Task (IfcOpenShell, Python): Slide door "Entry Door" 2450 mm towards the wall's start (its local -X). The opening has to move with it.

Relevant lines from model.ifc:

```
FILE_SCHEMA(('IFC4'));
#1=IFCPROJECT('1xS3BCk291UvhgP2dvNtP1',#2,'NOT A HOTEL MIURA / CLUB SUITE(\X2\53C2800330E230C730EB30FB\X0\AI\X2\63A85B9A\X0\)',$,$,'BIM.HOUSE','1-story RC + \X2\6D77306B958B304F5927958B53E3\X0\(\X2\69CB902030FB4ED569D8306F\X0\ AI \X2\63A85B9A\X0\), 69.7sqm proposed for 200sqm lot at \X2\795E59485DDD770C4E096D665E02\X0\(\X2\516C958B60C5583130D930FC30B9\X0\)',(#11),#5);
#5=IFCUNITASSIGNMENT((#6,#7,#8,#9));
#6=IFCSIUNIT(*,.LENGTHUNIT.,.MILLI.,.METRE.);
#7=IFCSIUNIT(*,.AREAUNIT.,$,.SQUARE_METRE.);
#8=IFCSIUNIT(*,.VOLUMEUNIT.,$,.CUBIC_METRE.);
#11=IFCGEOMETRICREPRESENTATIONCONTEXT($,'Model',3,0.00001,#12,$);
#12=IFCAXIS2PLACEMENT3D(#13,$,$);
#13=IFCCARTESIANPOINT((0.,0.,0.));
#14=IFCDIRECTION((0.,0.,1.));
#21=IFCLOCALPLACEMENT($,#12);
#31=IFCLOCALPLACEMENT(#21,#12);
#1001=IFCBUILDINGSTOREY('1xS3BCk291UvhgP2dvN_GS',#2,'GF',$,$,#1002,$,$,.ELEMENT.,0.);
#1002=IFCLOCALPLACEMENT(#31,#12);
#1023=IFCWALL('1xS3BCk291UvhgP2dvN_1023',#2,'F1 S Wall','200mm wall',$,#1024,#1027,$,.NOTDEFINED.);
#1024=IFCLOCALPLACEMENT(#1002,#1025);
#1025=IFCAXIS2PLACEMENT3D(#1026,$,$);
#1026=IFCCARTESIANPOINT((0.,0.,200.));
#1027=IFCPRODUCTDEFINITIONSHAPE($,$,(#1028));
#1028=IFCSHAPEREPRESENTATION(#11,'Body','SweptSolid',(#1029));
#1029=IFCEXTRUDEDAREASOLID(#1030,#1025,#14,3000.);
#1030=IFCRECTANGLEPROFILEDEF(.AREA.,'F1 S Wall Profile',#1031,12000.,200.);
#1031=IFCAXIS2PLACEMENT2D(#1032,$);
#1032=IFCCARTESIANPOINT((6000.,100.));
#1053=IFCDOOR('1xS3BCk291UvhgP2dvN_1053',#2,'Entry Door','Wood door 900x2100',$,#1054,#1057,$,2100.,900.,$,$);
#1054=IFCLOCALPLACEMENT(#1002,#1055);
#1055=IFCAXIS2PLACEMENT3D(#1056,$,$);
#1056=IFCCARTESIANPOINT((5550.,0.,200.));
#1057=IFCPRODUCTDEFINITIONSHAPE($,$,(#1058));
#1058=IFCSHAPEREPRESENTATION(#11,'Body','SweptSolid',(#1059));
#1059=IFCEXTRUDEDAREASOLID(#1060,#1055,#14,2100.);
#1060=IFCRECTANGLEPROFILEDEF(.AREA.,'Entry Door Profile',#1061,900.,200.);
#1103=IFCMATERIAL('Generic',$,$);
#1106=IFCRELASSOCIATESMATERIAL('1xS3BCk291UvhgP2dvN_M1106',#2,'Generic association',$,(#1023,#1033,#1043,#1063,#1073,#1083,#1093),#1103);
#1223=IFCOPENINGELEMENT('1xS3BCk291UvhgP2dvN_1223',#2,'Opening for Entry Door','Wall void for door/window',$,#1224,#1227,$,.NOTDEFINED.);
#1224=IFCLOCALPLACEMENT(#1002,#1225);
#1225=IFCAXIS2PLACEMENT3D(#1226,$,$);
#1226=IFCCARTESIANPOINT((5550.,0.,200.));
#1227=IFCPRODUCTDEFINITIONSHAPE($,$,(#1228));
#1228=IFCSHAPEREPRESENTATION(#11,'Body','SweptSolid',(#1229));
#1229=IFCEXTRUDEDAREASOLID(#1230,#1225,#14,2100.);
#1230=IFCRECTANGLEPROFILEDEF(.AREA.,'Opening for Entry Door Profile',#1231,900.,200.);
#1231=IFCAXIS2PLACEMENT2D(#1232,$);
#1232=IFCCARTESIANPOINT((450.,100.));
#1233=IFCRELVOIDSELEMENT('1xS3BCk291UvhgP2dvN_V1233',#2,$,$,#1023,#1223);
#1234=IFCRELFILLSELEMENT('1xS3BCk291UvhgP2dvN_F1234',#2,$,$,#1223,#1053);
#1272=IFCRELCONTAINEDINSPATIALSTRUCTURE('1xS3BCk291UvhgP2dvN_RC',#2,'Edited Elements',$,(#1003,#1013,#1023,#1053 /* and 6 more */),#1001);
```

```python
import ifcopenshell
import ifcopenshell.api.geometry
import ifcopenshell.util.placement

model = ifcopenshell.open("model.ifc")

door = model.by_id(1053)
opening = door.FillsVoids[0].RelatingOpeningElement
wall = opening.VoidsElements[0].RelatingBuildingElement

wall_matrix = ifcopenshell.util.placement.get_local_placement(wall.ObjectPlacement)
shift = wall_matrix[:3, 0] * -2450.0
before = ifcopenshell.util.placement.get_local_placement(door.ObjectPlacement)[:3, 3].copy()

# The door is not placed relative to its opening, so move both.
for product in (opening, door):
    matrix = ifcopenshell.util.placement.get_local_placement(product.ObjectPlacement)
    matrix[:3, 3] += shift
    ifcopenshell.api.geometry.edit_object_placement(model, product=product, matrix=matrix, is_si=False)

after = ifcopenshell.util.placement.get_local_placement(door.ObjectPlacement)[:3, 3]
print("door moved by", (after - before).round(3) + 0.0)

model.write("model_v2.ifc")
```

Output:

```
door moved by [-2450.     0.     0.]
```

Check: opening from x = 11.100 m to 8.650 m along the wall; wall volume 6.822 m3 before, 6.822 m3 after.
